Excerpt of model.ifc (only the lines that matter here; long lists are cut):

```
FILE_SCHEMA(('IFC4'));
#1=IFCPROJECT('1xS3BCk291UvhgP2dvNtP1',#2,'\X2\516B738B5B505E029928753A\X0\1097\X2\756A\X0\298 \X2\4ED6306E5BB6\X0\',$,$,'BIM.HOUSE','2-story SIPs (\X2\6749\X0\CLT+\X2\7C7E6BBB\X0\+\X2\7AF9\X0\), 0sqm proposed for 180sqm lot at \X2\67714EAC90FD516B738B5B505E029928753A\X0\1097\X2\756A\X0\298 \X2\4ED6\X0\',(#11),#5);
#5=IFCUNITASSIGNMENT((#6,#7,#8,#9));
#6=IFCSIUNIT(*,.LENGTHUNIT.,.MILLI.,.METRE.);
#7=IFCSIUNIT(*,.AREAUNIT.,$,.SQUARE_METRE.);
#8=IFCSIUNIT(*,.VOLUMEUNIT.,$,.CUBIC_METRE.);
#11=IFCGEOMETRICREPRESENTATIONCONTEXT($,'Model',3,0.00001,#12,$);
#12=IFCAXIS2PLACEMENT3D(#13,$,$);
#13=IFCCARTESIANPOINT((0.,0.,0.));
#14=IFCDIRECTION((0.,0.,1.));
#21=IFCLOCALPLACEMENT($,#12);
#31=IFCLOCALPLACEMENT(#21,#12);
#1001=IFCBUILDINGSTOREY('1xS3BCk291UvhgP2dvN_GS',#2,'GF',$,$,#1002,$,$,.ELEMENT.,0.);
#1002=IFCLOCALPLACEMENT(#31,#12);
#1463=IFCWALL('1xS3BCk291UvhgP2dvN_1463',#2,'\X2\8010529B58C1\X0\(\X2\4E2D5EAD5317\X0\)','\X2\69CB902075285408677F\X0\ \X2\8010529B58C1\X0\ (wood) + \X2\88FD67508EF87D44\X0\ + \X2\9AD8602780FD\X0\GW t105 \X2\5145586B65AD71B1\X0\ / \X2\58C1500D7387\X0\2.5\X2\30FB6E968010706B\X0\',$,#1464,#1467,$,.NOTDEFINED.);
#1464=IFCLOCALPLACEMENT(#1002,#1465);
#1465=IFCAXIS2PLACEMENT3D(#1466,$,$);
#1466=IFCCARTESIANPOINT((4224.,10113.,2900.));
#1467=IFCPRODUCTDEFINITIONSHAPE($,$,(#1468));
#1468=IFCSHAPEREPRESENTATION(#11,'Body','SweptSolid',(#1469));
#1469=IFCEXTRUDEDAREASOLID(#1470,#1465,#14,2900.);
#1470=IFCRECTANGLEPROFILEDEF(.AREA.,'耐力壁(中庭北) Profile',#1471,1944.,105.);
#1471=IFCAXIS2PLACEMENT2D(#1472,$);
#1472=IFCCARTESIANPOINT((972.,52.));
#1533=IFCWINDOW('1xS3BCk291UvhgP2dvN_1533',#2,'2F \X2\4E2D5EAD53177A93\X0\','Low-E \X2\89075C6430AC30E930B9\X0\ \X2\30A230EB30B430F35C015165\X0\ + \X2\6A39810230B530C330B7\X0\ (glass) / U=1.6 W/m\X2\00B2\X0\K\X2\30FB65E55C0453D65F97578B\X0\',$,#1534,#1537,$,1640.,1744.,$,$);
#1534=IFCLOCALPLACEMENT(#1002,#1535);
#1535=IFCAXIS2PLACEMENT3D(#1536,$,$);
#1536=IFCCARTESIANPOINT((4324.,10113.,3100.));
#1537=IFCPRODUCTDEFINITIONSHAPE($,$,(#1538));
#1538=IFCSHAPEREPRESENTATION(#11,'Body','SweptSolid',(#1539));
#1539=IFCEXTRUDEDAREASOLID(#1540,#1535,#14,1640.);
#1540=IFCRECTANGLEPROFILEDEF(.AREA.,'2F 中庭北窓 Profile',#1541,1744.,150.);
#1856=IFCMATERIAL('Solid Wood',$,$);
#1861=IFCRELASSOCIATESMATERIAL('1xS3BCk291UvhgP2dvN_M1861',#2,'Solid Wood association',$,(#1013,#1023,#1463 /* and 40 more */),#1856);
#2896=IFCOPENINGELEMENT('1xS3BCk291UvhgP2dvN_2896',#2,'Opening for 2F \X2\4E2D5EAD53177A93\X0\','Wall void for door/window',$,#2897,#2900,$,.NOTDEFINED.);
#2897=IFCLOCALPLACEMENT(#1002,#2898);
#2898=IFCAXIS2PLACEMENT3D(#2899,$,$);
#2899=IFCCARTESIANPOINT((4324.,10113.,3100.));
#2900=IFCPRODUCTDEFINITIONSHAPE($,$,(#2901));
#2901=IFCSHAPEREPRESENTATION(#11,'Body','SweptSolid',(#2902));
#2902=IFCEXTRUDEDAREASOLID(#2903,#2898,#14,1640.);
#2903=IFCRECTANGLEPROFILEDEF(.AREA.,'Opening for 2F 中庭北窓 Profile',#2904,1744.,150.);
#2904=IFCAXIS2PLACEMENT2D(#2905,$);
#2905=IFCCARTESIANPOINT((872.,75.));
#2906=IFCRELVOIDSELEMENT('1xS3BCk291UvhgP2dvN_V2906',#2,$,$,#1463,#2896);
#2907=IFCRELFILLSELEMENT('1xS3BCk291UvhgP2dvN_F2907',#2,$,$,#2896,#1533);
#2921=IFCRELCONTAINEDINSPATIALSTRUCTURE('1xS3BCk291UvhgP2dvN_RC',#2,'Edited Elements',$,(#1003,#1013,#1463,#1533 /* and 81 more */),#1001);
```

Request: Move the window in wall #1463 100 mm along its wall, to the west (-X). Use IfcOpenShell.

```python
import ifcopenshell
import ifcopenshell.api.geometry
import ifcopenshell.util.placement
import ifcopenshell.util.unit

model = ifcopenshell.open("model.ifc")
unit_scale = ifcopenshell.util.unit.calculate_unit_scale(model)

window = model.by_id(1533)
opening = window.FillsVoids[0].RelatingOpeningElement
wall = opening.VoidsElements[0].RelatingBuildingElement

wall_matrix = ifcopenshell.util.placement.get_local_placement(wall.ObjectPlacement)
shift = wall_matrix[:3, 0] * -0.1 / unit_scale
before = ifcopenshell.util.placement.get_local_placement(window.ObjectPlacement)[:3, 3].copy()

# The window is not placed relative to its opening, so move both.
for product in (opening, window):
    matrix = ifcopenshell.util.placement.get_local_placement(product.ObjectPlacement)
    matrix[:3, 3] += shift
    ifcopenshell.api.geometry.edit_object_placement(model, product=product, matrix=matrix, is_si=False)

after = ifcopenshell.util.placement.get_local_placement(window.ObjectPlacement)[:3, 3]
print("window moved by", (after - before).round(3) + 0.0)

model.write("model_edited.ifc")
```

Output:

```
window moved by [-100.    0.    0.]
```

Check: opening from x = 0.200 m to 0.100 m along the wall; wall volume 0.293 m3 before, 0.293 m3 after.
